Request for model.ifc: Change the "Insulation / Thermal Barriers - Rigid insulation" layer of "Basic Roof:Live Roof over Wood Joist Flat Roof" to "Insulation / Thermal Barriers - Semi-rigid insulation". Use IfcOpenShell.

First a look at what the model holds.

```python
import ifcopenshell
import ifcopenshell.util.element

model = ifcopenshell.open("model.ifc")
print(model.schema)
for layer_set in model.by_type("IfcMaterialLayerSet"):
    if layer_set.LayerSetName == "Basic Roof:Live Roof over Wood Joist Flat Roof":
        for layer in layer_set.MaterialLayers:
            print(layer.id(), layer.Material and layer.Material.Name, layer.LayerThickness, sep=" | ")
        print(len(ifcopenshell.util.element.get_elements_by_material(model, layer_set)), "elements and types use it")
print(sorted(m.Name for m in model.by_type("IfcMaterial") if m.Name)[:60])
```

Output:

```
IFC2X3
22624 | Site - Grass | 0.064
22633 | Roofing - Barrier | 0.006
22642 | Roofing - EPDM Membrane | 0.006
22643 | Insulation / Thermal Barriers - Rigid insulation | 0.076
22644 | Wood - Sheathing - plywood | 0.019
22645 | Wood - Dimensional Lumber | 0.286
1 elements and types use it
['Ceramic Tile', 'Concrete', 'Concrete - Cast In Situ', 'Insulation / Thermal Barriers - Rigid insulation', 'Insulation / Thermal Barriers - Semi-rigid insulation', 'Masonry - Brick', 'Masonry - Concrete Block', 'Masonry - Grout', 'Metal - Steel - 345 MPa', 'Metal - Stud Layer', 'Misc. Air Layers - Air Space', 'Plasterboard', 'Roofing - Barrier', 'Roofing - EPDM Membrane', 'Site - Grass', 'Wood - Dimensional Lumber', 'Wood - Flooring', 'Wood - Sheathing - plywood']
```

```python
import ifcopenshell
import ifcopenshell.api.material

model = ifcopenshell.open("model.ifc")

layer_set = next(s for s in model.by_type("IfcMaterialLayerSet") if s.LayerSetName == "Basic Roof:Live Roof over Wood Joist Flat Roof")
layer = next(l for l in layer_set.MaterialLayers if l.Material and l.Material.Name == "Insulation / Thermal Barriers - Rigid insulation")
material = next(m for m in model.by_type("IfcMaterial") if m.Name == "Insulation / Thermal Barriers - Semi-rigid insulation")

# Point this one layer at the other material; renaming the old one would change it everywhere.
ifcopenshell.api.material.edit_layer(model, layer=layer, attributes={}, material=material)

print([l.Material.Name if l.Material else None for l in layer_set.MaterialLayers])

model.write("model-out.ifc")
```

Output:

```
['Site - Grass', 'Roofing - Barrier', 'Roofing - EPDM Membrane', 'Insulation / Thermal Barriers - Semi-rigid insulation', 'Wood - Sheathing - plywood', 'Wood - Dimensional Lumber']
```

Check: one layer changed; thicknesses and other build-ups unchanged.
